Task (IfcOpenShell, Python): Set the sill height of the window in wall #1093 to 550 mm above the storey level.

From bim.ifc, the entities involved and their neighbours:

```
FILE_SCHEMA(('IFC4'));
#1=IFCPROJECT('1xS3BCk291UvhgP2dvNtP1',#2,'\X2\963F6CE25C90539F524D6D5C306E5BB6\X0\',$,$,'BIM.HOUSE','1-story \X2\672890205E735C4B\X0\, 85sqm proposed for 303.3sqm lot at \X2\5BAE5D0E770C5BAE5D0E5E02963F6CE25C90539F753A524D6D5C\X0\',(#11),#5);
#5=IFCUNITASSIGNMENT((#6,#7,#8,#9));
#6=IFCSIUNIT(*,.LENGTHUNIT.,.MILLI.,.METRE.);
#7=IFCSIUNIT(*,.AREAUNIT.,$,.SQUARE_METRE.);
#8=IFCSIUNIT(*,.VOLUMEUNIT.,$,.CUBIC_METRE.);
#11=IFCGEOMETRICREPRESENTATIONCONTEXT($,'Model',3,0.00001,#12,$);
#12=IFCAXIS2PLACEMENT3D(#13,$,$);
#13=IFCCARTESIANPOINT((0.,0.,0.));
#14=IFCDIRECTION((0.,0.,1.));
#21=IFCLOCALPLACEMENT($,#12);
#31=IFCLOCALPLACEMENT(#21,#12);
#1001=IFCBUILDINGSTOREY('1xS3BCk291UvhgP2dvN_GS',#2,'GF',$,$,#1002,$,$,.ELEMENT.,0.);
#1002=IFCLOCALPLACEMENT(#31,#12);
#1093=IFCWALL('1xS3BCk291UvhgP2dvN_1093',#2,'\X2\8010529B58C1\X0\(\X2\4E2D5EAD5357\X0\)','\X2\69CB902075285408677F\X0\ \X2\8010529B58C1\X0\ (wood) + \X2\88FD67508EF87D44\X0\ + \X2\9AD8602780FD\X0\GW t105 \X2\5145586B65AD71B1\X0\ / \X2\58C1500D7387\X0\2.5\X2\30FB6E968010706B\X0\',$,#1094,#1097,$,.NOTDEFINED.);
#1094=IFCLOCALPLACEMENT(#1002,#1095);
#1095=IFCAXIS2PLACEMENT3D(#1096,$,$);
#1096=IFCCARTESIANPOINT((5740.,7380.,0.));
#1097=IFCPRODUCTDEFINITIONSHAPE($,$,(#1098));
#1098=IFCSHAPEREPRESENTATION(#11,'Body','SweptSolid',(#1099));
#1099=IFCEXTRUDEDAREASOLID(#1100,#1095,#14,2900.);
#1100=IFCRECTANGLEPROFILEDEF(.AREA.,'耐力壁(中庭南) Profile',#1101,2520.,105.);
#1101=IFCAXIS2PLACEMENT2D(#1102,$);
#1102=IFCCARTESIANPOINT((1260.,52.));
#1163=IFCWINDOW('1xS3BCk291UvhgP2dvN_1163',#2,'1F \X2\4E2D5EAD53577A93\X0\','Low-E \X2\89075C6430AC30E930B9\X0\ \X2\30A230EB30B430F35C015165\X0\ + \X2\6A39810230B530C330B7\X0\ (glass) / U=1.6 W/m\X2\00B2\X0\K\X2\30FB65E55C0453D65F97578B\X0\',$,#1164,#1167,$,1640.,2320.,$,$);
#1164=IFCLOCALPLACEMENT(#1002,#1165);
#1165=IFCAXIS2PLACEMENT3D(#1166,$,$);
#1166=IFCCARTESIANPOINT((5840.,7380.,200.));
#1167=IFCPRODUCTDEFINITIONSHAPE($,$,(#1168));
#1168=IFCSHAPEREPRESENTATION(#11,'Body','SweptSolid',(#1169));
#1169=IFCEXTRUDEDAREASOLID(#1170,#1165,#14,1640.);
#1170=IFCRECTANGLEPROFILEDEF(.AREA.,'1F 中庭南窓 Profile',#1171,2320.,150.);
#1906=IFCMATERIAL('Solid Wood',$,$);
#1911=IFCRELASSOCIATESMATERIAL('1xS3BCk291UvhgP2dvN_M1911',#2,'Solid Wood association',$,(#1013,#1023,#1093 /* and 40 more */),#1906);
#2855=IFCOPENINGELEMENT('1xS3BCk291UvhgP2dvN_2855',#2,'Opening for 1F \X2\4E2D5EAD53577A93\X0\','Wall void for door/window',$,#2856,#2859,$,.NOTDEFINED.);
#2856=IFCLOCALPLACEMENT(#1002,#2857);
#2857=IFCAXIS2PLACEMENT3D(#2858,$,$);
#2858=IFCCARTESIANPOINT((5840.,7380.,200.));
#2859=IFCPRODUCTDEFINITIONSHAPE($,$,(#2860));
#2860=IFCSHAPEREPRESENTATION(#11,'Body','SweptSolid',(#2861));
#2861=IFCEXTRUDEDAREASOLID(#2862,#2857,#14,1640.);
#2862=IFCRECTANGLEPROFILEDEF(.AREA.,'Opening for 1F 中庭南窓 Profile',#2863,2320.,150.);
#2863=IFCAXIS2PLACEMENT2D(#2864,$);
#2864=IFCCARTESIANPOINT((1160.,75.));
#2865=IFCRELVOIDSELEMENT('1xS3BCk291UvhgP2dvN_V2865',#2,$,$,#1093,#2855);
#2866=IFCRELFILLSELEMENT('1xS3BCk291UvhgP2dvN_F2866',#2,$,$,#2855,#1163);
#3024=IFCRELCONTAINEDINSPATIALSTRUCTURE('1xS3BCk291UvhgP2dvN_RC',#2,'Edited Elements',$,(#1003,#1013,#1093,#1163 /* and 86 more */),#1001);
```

```python
import numpy as np
import ifcopenshell
import ifcopenshell.api.geometry
import ifcopenshell.geom
import ifcopenshell.util.element
import ifcopenshell.util.placement
import ifcopenshell.util.shape
import ifcopenshell.util.unit

model = ifcopenshell.open("bim.ifc")
unit_scale = ifcopenshell.util.unit.calculate_unit_scale(model)

window = model.by_guid("1xS3BCk291UvhgP2dvN_1163")
opening = window.FillsVoids[0].RelatingOpeningElement
storey = ifcopenshell.util.element.get_container(window, ifc_class="IfcBuildingStorey")
level = ifcopenshell.util.placement.get_local_placement(storey.ObjectPlacement)[2, 3]

# The opening's origin need not be at the sill, so measure its lowest point.
shape = ifcopenshell.geom.create_shape(ifcopenshell.geom.settings(), opening)
bottom = ifcopenshell.util.shape.get_shape_bottom_elevation(shape, shape.geometry) / unit_scale
dz = level + 550.0 - bottom

shift = np.array([0.0, 0.0, dz])
# The window is not placed relative to its opening, so move both.
for product in (opening, window):
    matrix = ifcopenshell.util.placement.get_local_placement(product.ObjectPlacement)
    matrix[:3, 3] += shift
    ifcopenshell.api.geometry.edit_object_placement(model, product=product, matrix=matrix, is_si=False)

print(f"moved by {dz * unit_scale:+.3f} m")

model.write("bim_edited.ifc")
```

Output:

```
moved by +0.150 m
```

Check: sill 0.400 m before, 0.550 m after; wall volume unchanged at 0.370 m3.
